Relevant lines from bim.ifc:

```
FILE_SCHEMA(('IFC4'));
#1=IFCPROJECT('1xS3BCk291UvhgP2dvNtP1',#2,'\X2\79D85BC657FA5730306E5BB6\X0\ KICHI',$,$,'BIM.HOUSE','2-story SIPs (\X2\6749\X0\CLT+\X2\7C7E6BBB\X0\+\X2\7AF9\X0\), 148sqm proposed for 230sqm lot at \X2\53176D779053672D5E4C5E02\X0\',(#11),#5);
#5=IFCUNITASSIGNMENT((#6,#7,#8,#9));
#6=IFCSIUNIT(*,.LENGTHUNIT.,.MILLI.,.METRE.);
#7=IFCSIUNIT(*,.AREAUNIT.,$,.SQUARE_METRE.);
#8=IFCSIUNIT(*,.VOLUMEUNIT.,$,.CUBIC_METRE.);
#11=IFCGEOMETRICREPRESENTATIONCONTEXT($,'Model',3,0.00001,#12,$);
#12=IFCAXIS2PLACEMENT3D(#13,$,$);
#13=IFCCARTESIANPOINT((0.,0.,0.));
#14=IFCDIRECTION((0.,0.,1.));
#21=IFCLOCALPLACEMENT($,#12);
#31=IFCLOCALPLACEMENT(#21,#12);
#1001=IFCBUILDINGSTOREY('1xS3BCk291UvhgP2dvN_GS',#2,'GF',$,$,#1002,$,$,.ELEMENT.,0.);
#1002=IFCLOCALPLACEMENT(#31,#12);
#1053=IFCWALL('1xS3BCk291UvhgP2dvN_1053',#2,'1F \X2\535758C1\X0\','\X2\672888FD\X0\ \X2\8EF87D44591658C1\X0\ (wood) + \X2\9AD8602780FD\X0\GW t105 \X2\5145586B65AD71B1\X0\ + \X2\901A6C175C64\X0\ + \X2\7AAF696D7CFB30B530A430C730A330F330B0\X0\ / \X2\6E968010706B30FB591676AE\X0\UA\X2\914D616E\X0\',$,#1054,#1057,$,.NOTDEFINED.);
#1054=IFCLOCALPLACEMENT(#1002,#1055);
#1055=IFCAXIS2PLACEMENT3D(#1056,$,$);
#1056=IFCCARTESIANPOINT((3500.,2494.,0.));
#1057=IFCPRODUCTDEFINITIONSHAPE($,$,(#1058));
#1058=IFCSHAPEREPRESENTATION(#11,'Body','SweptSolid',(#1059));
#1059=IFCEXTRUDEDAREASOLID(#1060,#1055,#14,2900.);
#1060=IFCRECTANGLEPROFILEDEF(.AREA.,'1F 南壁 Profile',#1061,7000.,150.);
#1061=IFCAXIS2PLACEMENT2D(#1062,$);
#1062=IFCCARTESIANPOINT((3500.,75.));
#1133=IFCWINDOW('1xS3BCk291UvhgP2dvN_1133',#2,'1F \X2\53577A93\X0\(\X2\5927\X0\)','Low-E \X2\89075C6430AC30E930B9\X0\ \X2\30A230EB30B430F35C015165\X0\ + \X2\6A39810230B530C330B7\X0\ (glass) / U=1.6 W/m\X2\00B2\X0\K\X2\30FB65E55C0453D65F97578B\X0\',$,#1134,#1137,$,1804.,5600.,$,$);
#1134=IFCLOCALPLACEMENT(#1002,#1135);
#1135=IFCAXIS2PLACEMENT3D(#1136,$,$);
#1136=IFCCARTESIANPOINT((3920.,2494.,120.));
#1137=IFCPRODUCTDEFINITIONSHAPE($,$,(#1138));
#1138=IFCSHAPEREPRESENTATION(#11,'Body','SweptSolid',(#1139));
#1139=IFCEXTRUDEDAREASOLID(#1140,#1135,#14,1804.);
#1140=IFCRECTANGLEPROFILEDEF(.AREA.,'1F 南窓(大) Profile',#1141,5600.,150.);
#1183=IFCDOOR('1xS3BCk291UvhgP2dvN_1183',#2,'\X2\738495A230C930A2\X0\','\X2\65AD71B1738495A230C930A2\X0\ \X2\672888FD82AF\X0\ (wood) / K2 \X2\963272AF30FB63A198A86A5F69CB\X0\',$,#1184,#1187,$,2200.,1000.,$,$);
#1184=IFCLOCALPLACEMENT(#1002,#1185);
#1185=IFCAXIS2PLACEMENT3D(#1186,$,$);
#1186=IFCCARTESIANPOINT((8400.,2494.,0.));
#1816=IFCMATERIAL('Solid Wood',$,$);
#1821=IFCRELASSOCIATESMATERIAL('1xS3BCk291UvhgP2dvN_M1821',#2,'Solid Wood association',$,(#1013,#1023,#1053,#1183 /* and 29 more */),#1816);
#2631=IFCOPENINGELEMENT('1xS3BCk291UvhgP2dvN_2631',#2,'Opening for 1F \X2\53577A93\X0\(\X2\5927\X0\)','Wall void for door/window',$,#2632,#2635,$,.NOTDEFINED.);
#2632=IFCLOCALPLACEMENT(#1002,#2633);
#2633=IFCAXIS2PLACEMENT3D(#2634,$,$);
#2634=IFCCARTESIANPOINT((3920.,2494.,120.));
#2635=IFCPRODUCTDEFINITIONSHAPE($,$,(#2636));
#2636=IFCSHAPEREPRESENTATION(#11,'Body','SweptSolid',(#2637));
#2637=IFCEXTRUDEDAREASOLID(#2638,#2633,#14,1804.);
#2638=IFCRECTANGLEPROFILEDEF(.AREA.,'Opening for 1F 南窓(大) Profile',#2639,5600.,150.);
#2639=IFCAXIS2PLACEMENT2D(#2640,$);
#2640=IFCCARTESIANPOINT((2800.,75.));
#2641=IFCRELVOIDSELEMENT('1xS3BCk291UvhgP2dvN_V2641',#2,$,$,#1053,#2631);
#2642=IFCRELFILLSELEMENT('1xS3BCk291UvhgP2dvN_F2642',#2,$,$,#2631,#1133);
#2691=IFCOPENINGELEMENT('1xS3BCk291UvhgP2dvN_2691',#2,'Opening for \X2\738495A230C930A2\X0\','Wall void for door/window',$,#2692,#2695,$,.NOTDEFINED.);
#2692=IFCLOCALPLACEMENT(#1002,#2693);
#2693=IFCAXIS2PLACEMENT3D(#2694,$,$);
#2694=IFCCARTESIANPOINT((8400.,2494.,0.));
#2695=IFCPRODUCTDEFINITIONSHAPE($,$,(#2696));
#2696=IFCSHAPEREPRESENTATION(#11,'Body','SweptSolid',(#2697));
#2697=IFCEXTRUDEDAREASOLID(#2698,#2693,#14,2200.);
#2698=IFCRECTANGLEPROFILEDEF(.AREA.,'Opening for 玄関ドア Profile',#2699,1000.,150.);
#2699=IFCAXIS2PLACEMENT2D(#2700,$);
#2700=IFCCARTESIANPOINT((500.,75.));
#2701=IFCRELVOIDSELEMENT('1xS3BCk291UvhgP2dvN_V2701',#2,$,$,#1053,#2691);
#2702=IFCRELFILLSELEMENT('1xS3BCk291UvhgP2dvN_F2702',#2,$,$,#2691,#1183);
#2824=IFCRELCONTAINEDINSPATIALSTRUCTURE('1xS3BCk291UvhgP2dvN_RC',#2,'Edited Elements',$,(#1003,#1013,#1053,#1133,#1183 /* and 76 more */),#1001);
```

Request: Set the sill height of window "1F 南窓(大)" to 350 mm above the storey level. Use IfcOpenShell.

```python
import numpy as np
import ifcopenshell
import ifcopenshell.api.geometry
import ifcopenshell.geom
import ifcopenshell.util.element
import ifcopenshell.util.placement
import ifcopenshell.util.shape
import ifcopenshell.util.unit

model = ifcopenshell.open("bim.ifc")
unit_scale = ifcopenshell.util.unit.calculate_unit_scale(model)

window = model.by_guid("1xS3BCk291UvhgP2dvN_1133")
opening = window.FillsVoids[0].RelatingOpeningElement
storey = ifcopenshell.util.element.get_container(window, ifc_class="IfcBuildingStorey")
level = ifcopenshell.util.placement.get_local_placement(storey.ObjectPlacement)[2, 3]

# The opening's origin need not be at the sill, so measure its lowest point.
shape = ifcopenshell.geom.create_shape(ifcopenshell.geom.settings(), opening)
bottom = ifcopenshell.util.shape.get_shape_bottom_elevation(shape, shape.geometry) / unit_scale
dz = level + 0.35 / unit_scale - bottom

shift = np.array([0.0, 0.0, dz])
# The window is not placed relative to its opening, so move both.
for product in (opening, window):
    matrix = ifcopenshell.util.placement.get_local_placement(product.ObjectPlacement)
    matrix[:3, 3] += shift
    ifcopenshell.api.geometry.edit_object_placement(model, product=product, matrix=matrix, is_si=False)

print(f"moved by {dz * unit_scale:+.3f} m")

model.write("bim-out.ifc")
```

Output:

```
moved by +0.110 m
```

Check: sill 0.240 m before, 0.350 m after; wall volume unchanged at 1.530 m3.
